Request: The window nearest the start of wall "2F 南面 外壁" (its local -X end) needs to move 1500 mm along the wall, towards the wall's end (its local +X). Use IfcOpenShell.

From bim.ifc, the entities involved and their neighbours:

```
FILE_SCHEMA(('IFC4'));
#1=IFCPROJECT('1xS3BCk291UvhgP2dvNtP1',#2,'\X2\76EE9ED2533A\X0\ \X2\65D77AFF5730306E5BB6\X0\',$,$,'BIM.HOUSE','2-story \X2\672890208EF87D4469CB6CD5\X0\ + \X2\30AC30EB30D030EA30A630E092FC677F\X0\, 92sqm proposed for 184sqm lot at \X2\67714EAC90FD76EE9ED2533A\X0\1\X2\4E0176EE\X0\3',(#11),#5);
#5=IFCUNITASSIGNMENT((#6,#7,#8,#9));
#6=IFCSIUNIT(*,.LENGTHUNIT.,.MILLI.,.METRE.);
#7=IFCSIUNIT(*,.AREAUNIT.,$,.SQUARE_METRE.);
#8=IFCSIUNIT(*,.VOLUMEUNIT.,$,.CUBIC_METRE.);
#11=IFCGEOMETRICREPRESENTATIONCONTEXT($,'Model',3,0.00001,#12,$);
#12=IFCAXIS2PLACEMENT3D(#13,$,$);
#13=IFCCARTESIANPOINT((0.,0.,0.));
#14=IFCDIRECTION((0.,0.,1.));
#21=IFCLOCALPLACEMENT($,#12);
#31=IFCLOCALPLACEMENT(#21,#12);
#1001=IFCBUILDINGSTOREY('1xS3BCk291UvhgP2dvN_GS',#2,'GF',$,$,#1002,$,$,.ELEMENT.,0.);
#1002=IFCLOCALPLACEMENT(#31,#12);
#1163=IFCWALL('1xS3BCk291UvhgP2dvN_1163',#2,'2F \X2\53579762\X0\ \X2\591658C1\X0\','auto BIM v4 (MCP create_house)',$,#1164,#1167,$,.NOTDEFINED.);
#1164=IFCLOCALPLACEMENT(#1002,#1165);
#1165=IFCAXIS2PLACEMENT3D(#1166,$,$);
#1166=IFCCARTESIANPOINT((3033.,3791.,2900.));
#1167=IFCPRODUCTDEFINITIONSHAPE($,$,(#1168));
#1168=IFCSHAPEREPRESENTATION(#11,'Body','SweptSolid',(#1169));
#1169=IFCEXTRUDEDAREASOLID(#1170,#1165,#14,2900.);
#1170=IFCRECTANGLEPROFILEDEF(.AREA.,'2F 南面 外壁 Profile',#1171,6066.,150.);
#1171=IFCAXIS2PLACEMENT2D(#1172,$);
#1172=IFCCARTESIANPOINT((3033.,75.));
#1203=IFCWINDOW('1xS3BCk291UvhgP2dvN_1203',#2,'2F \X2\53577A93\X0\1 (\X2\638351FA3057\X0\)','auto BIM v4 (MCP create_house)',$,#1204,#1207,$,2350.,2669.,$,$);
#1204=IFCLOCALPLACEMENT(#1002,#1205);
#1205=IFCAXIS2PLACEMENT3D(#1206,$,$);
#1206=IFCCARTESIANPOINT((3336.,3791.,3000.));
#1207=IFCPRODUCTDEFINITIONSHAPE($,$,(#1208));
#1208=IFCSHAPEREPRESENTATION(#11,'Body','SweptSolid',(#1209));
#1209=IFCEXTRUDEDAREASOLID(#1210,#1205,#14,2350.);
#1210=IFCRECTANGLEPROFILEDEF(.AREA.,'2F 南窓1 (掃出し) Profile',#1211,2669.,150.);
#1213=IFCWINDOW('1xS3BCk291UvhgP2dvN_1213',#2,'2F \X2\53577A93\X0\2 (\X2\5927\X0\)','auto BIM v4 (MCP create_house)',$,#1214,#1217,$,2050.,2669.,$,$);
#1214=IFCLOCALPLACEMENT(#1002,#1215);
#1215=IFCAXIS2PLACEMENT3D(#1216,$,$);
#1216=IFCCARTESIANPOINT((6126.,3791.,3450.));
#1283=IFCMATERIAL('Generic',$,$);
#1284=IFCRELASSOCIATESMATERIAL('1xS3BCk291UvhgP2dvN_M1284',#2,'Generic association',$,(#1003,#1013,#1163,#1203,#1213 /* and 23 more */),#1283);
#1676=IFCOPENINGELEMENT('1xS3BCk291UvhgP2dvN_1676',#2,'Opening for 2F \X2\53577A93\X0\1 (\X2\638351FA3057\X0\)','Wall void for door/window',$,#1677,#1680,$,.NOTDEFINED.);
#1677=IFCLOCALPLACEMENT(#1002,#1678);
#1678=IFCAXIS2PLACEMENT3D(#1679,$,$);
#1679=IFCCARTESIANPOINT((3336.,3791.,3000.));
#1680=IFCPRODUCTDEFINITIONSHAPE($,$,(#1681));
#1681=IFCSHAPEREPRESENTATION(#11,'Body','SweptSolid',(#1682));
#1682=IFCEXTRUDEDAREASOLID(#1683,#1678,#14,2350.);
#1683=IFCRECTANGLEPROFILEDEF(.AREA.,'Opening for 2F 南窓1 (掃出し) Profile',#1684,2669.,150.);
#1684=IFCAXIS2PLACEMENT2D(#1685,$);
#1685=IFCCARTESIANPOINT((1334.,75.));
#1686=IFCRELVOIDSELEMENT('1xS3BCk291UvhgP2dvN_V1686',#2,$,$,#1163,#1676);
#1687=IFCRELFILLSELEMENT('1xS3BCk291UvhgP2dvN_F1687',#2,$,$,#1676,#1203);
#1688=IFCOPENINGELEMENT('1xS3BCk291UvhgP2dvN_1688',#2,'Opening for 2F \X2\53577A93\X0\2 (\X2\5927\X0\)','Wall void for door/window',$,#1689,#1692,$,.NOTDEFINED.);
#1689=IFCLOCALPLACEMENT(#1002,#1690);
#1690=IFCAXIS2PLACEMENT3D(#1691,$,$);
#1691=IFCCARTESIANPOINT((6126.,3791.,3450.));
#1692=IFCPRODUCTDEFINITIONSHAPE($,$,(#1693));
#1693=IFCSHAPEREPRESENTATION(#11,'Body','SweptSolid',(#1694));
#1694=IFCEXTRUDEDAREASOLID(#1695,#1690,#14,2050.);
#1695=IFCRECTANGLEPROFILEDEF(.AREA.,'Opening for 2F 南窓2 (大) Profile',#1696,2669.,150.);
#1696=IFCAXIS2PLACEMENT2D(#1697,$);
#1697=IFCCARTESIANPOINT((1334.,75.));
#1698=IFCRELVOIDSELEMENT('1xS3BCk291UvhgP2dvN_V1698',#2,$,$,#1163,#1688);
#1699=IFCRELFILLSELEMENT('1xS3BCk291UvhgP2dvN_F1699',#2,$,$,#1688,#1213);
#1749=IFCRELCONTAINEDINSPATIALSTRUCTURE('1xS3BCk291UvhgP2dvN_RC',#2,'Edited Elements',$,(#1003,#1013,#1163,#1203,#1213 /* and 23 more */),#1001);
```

```python
import ifcopenshell
import ifcopenshell.api.geometry
import ifcopenshell.util.placement
import ifcopenshell.util.unit

model = ifcopenshell.open("bim.ifc")
unit_scale = ifcopenshell.util.unit.calculate_unit_scale(model)

window = model.by_guid("1xS3BCk291UvhgP2dvN_1203")
opening = window.FillsVoids[0].RelatingOpeningElement
wall = opening.VoidsElements[0].RelatingBuildingElement

wall_matrix = ifcopenshell.util.placement.get_local_placement(wall.ObjectPlacement)
shift = wall_matrix[:3, 0] * 1.5 / unit_scale
before = ifcopenshell.util.placement.get_local_placement(window.ObjectPlacement)[:3, 3].copy()

# The window is not placed relative to its opening, so move both.
for product in (opening, window):
    matrix = ifcopenshell.util.placement.get_local_placement(product.ObjectPlacement)
    matrix[:3, 3] += shift
    ifcopenshell.api.geometry.edit_object_placement(model, product=product, matrix=matrix, is_si=False)

after = ifcopenshell.util.placement.get_local_placement(window.ObjectPlacement)[:3, 3]
print("window moved by", (after - before).round(3) + 0.0)

model.write("bim_rev.ifc")
```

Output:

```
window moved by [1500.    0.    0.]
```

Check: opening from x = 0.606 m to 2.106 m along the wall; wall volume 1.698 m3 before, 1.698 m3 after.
